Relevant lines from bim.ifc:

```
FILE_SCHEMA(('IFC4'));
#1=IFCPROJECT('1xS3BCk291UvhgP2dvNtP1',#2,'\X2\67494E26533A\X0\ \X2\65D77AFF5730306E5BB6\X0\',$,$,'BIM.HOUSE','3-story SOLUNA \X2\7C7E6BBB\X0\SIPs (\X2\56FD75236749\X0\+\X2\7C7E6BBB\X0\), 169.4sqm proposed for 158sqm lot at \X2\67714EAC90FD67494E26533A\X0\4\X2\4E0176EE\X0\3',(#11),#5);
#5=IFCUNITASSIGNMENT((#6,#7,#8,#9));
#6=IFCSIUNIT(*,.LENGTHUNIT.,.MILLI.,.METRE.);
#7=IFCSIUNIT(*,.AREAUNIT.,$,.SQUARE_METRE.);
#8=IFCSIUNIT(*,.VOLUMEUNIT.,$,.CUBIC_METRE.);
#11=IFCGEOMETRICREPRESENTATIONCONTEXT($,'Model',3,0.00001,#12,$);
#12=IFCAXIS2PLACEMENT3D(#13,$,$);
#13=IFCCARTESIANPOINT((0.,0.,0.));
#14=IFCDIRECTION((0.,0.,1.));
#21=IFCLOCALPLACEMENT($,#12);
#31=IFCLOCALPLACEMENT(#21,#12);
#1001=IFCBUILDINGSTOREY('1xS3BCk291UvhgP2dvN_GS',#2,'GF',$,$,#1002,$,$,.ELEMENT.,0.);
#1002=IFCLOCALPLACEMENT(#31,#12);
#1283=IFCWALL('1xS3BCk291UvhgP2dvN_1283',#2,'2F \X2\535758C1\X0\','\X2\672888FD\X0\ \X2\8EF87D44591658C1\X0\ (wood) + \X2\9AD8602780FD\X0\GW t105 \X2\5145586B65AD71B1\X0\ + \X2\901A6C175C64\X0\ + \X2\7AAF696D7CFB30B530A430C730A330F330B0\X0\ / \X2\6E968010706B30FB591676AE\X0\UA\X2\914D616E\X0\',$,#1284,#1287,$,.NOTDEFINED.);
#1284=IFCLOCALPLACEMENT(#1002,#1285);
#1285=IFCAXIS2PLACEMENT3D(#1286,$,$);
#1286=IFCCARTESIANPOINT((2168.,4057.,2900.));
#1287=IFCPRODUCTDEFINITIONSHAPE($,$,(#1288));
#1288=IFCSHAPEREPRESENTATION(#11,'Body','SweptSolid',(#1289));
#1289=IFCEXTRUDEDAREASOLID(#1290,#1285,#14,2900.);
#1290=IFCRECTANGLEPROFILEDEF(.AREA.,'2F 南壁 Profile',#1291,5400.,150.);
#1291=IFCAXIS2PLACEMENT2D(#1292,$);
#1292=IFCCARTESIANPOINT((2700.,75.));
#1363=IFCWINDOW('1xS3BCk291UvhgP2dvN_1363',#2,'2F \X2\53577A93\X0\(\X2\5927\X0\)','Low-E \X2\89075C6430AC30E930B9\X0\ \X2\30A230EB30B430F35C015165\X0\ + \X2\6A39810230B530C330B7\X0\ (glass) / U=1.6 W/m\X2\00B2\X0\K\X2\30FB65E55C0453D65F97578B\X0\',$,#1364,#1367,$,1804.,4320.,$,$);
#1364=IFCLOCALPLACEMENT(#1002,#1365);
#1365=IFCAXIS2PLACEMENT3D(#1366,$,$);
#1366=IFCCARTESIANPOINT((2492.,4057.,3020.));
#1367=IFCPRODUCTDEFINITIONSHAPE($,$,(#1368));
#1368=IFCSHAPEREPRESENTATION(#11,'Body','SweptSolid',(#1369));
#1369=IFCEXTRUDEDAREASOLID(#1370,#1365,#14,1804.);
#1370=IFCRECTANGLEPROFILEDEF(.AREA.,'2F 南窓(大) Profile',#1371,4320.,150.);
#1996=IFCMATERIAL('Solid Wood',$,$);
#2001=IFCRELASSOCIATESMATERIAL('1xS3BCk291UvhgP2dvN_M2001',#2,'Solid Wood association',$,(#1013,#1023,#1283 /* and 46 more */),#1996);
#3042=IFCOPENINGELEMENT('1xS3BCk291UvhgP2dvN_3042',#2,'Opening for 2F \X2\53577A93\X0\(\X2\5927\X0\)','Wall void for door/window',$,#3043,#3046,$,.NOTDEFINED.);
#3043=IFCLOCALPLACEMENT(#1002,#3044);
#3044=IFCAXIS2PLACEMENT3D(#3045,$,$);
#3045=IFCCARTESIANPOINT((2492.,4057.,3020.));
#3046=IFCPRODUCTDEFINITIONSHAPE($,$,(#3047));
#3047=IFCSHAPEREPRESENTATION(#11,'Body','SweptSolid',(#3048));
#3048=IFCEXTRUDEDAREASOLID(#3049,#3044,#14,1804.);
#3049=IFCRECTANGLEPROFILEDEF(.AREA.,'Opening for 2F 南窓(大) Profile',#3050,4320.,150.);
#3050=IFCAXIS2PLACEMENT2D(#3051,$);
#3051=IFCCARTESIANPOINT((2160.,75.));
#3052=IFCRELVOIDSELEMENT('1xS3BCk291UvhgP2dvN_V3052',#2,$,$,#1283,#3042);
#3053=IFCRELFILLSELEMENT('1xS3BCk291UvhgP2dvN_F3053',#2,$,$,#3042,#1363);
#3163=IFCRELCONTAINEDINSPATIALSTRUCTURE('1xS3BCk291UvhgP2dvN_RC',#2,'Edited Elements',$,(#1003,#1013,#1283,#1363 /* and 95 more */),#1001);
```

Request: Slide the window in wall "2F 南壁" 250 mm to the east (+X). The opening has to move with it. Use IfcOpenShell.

```python
import ifcopenshell
import ifcopenshell.api.geometry
import ifcopenshell.util.placement
import ifcopenshell.util.unit

model = ifcopenshell.open("bim.ifc")
unit_scale = ifcopenshell.util.unit.calculate_unit_scale(model)

window = model.by_id(1363)
opening = window.FillsVoids[0].RelatingOpeningElement
wall = opening.VoidsElements[0].RelatingBuildingElement

wall_matrix = ifcopenshell.util.placement.get_local_placement(wall.ObjectPlacement)
shift = wall_matrix[:3, 0] * 0.25 / unit_scale
before = ifcopenshell.util.placement.get_local_placement(window.ObjectPlacement)[:3, 3].copy()

# The window is not placed relative to its opening, so move both.
for product in (opening, window):
    matrix = ifcopenshell.util.placement.get_local_placement(product.ObjectPlacement)
    matrix[:3, 3] += shift
    ifcopenshell.api.geometry.edit_object_placement(model, product=product, matrix=matrix, is_si=False)

after = ifcopenshell.util.placement.get_local_placement(window.ObjectPlacement)[:3, 3]
print("window moved by", (after - before).round(3) + 0.0)

model.write("bim_v2.ifc")
```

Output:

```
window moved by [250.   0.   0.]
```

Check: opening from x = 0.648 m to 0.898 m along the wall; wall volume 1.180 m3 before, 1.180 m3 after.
